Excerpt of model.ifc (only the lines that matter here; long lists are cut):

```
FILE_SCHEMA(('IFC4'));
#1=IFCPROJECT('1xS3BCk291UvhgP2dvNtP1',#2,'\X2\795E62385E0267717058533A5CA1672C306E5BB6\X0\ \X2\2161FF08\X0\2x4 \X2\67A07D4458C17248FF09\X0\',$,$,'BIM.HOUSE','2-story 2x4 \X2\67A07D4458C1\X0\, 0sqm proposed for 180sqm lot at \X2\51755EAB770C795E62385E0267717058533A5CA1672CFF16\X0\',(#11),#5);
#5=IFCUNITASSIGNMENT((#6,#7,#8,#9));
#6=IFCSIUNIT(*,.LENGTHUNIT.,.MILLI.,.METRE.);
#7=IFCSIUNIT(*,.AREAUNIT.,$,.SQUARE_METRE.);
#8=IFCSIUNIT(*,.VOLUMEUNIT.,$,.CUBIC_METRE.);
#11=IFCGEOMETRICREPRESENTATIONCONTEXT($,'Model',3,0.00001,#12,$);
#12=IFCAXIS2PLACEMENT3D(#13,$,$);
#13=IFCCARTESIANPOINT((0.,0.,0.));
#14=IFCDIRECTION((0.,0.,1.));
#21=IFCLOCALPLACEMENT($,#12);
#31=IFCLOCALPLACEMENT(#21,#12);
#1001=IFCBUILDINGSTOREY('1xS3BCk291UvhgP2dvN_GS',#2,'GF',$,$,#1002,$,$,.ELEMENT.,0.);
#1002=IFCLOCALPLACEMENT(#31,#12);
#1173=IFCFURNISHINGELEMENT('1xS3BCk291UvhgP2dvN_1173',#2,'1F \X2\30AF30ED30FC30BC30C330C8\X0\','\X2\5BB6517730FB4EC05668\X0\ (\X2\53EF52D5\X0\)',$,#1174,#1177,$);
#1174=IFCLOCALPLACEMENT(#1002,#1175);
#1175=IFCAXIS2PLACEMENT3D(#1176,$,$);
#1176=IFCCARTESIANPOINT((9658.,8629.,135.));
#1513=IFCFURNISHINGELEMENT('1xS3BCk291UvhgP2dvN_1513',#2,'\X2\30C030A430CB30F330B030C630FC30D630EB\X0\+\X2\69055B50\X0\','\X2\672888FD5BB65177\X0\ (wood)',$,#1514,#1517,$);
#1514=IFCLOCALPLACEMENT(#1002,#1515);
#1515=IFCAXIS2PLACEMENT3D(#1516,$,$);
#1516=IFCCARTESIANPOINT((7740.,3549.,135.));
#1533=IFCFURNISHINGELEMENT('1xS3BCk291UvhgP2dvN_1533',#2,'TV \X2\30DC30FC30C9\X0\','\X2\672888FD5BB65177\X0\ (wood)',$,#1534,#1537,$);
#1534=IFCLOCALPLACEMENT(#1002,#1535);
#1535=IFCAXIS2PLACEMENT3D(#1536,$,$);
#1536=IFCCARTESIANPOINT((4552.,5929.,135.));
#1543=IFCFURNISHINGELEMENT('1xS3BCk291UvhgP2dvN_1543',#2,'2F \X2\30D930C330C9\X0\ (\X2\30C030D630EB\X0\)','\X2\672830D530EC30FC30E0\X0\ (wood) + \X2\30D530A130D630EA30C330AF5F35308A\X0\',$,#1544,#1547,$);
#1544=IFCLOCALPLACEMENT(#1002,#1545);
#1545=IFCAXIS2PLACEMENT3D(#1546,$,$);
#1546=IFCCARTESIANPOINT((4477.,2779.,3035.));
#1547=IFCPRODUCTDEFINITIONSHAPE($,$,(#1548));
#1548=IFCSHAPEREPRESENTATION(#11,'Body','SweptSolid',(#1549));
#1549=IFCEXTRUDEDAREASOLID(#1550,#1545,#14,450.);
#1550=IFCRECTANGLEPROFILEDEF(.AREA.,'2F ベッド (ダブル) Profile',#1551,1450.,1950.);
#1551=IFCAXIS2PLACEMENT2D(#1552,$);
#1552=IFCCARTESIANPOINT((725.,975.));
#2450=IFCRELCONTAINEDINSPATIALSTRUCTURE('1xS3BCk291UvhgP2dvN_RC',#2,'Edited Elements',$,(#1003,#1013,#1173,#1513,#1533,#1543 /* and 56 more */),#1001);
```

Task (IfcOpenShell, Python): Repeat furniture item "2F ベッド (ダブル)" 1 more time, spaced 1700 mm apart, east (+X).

```python
import numpy as np
import ifcopenshell
import ifcopenshell.api.geometry
import ifcopenshell.api.root
import ifcopenshell.util.element
import ifcopenshell.util.placement
import ifcopenshell.util.unit

model = ifcopenshell.open("model.ifc")
unit_scale = ifcopenshell.util.unit.calculate_unit_scale(model)


def reuse_history(source, copy):
    """copy_class also copies each property set's owner history, people and application; keep the originals."""
    for rel in copy.IsDefinedBy:
        if rel.is_a("IfcRelDefinesByProperties") and (history := rel.RelatingPropertyDefinition.OwnerHistory):
            rel.RelatingPropertyDefinition.OwnerHistory = source.OwnerHistory
            ifcopenshell.util.element.remove_deep2(model, history)


source = model.by_guid("1xS3BCk291UvhgP2dvN_1543")
base = ifcopenshell.util.placement.get_local_placement(source.ObjectPlacement)
step = np.array([1.0, 0.0, 0.0]) * 1.7 / unit_scale

for i in range(1, 2):
    copy = ifcopenshell.api.root.copy_class(model, product=source)
    copy.Representation = ifcopenshell.util.element.copy_deep(
        model, source.Representation, exclude=["IfcGeometricRepresentationContext", "IfcRepresentationMap"]
    )
    reuse_history(source, copy)
    matrix = base.copy()
    matrix[:3, 3] += i * step
    print("added at", matrix[:3, 3].round(3) + 0.0)
    ifcopenshell.api.geometry.edit_object_placement(model, product=copy, matrix=matrix, is_si=False)

model.write("model_updated.ifc")
```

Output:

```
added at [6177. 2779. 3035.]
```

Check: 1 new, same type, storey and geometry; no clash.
